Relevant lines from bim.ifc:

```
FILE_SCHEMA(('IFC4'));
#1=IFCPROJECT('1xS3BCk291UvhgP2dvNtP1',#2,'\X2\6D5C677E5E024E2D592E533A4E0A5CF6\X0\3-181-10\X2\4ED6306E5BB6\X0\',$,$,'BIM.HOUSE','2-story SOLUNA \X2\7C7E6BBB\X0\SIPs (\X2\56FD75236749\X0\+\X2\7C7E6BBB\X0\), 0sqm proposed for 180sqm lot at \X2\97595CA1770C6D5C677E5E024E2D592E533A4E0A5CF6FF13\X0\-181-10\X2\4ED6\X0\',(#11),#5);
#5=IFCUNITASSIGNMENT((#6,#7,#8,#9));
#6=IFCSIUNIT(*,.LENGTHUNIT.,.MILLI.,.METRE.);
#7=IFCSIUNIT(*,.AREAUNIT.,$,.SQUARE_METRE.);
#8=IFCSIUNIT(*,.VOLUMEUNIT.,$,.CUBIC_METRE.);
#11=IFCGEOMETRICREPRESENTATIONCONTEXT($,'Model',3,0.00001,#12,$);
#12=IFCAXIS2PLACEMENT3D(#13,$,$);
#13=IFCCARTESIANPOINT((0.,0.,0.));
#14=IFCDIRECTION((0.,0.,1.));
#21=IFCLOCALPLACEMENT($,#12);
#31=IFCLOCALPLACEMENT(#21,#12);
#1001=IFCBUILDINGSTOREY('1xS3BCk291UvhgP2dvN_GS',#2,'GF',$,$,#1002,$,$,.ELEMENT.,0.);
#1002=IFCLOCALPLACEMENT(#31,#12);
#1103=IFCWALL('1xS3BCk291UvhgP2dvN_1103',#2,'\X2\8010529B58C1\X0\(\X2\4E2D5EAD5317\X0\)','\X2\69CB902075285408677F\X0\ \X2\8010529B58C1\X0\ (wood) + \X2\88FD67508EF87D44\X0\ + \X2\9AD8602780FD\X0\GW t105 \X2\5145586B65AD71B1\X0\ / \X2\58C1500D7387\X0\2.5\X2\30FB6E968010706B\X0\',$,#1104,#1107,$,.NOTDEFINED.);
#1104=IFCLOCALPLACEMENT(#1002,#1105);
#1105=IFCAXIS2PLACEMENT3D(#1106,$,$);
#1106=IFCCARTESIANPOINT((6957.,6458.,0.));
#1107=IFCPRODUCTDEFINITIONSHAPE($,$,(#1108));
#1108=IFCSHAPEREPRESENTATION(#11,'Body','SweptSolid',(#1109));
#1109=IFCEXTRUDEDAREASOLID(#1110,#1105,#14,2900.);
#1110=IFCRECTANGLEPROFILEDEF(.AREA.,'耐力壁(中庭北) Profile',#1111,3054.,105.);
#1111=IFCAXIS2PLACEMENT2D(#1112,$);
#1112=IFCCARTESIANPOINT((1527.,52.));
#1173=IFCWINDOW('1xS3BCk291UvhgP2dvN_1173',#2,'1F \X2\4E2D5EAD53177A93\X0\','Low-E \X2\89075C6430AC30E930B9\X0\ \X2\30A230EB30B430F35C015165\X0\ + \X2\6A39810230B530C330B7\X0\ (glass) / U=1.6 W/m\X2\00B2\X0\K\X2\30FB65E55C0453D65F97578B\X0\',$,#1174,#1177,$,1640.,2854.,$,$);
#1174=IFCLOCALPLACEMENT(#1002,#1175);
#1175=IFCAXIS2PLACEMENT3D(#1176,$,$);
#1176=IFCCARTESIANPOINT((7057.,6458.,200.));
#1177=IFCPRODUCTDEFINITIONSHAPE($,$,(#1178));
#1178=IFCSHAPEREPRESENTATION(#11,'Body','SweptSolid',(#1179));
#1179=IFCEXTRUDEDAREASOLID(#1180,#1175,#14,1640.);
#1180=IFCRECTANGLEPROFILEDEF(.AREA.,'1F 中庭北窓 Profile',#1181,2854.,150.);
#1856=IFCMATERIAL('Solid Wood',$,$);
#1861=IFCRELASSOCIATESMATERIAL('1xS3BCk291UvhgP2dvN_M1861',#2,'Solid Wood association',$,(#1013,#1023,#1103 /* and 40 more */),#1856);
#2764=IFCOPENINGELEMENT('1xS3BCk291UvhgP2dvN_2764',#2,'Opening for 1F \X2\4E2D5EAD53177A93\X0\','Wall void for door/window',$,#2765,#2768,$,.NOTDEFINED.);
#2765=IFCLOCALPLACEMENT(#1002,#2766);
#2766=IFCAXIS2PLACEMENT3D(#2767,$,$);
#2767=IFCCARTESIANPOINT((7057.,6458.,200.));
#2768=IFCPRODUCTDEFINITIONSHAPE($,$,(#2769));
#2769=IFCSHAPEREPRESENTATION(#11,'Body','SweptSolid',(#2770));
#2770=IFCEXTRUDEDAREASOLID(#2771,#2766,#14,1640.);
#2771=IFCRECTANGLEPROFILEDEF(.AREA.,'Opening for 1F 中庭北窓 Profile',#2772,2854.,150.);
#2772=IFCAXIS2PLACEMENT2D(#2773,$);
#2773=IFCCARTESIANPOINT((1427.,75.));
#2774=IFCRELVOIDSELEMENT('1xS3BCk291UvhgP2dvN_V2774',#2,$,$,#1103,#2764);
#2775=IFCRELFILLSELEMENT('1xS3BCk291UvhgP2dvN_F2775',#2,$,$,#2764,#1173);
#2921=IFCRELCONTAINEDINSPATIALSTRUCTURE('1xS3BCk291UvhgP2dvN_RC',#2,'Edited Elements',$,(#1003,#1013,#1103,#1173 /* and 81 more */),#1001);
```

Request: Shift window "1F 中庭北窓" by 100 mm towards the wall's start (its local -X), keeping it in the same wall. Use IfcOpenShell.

```python
import ifcopenshell
import ifcopenshell.api.geometry
import ifcopenshell.util.placement
import ifcopenshell.util.unit

model = ifcopenshell.open("bim.ifc")
unit_scale = ifcopenshell.util.unit.calculate_unit_scale(model)

window = model.by_guid("1xS3BCk291UvhgP2dvN_1173")
opening = window.FillsVoids[0].RelatingOpeningElement
wall = opening.VoidsElements[0].RelatingBuildingElement

wall_matrix = ifcopenshell.util.placement.get_local_placement(wall.ObjectPlacement)
shift = wall_matrix[:3, 0] * -0.1 / unit_scale
before = ifcopenshell.util.placement.get_local_placement(window.ObjectPlacement)[:3, 3].copy()

# The window is not placed relative to its opening, so move both.
for product in (opening, window):
    matrix = ifcopenshell.util.placement.get_local_placement(product.ObjectPlacement)
    matrix[:3, 3] += shift
    ifcopenshell.api.geometry.edit_object_placement(model, product=product, matrix=matrix, is_si=False)

after = ifcopenshell.util.placement.get_local_placement(window.ObjectPlacement)[:3, 3]
print("window moved by", (after - before).round(3) + 0.0)

model.write("bim_edited.ifc")
```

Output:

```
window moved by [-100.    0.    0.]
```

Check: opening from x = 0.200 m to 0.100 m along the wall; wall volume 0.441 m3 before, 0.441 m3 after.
